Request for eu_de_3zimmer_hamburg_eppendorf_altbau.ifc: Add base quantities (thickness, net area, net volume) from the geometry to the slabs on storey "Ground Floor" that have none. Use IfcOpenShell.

First a look at what the model holds.

```python
import ifcopenshell
import ifcopenshell.util.element
import ifcopenshell.util.unit

model = ifcopenshell.open("eu_de_3zimmer_hamburg_eppendorf_altbau.ifc")
print(model.schema)
for unit_type in ("LENGTHUNIT", "AREAUNIT", "VOLUMEUNIT"):
    print(unit_type, ifcopenshell.util.unit.calculate_unit_scale(model, unit_type))
storey = next(s for s in model.by_type("IfcBuildingStorey") if s.Name == "Ground Floor")
slabs = [e for e in ifcopenshell.util.element.get_decomposition(storey) if e.is_a("IfcSlab")]
for e in sorted(slabs, key=lambda e: e.id()):
    print(e.id(), e.is_a(), e.Name, list(ifcopenshell.util.element.get_psets(e, qtos_only=True)), sep=" | ")
```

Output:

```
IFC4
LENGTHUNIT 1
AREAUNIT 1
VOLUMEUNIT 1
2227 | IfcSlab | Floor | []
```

```python
import ifcopenshell
import ifcopenshell.api.pset
import ifcopenshell.geom
import ifcopenshell.util.element
import ifcopenshell.util.shape
import ifcopenshell.util.unit

model = ifcopenshell.open("eu_de_3zimmer_hamburg_eppendorf_altbau.ifc")
unit_scale = ifcopenshell.util.unit.calculate_unit_scale(model)
area_scale = ifcopenshell.util.unit.calculate_unit_scale(model, "AREAUNIT")
volume_scale = ifcopenshell.util.unit.calculate_unit_scale(model, "VOLUMEUNIT")
settings = ifcopenshell.geom.settings()

storey = next(s for s in model.by_type("IfcBuildingStorey") if s.Name == "Ground Floor")
slabs = [e for e in ifcopenshell.util.element.get_decomposition(storey) if e.is_a("IfcSlab")]

for e in sorted(slabs, key=lambda e: e.id()):
    if ifcopenshell.util.element.get_psets(e, qtos_only=True, should_inherit=False):
        continue
    # Geometry comes back in metres, in the element's own axes.
    shape = ifcopenshell.geom.create_shape(settings, e)
    values = {
        "Width": ifcopenshell.util.shape.get_z(shape.geometry) / unit_scale,
        "NetArea": ifcopenshell.util.shape.get_footprint_area(shape.geometry) / area_scale,
        "NetVolume": ifcopenshell.util.shape.get_volume(shape.geometry) / volume_scale,
    }
    qto = ifcopenshell.api.pset.add_qto(model, product=e, name="Qto_SlabBaseQuantities")
    ifcopenshell.api.pset.edit_qto(model, qto=qto, properties=values)
    print(e.id(), {k: round(v, 3) for k, v in values.items()})

model.write("eu_de_3zimmer_hamburg_eppendorf_altbau_updated.ifc")
```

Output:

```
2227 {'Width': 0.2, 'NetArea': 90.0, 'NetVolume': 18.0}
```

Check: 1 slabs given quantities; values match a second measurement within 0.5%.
